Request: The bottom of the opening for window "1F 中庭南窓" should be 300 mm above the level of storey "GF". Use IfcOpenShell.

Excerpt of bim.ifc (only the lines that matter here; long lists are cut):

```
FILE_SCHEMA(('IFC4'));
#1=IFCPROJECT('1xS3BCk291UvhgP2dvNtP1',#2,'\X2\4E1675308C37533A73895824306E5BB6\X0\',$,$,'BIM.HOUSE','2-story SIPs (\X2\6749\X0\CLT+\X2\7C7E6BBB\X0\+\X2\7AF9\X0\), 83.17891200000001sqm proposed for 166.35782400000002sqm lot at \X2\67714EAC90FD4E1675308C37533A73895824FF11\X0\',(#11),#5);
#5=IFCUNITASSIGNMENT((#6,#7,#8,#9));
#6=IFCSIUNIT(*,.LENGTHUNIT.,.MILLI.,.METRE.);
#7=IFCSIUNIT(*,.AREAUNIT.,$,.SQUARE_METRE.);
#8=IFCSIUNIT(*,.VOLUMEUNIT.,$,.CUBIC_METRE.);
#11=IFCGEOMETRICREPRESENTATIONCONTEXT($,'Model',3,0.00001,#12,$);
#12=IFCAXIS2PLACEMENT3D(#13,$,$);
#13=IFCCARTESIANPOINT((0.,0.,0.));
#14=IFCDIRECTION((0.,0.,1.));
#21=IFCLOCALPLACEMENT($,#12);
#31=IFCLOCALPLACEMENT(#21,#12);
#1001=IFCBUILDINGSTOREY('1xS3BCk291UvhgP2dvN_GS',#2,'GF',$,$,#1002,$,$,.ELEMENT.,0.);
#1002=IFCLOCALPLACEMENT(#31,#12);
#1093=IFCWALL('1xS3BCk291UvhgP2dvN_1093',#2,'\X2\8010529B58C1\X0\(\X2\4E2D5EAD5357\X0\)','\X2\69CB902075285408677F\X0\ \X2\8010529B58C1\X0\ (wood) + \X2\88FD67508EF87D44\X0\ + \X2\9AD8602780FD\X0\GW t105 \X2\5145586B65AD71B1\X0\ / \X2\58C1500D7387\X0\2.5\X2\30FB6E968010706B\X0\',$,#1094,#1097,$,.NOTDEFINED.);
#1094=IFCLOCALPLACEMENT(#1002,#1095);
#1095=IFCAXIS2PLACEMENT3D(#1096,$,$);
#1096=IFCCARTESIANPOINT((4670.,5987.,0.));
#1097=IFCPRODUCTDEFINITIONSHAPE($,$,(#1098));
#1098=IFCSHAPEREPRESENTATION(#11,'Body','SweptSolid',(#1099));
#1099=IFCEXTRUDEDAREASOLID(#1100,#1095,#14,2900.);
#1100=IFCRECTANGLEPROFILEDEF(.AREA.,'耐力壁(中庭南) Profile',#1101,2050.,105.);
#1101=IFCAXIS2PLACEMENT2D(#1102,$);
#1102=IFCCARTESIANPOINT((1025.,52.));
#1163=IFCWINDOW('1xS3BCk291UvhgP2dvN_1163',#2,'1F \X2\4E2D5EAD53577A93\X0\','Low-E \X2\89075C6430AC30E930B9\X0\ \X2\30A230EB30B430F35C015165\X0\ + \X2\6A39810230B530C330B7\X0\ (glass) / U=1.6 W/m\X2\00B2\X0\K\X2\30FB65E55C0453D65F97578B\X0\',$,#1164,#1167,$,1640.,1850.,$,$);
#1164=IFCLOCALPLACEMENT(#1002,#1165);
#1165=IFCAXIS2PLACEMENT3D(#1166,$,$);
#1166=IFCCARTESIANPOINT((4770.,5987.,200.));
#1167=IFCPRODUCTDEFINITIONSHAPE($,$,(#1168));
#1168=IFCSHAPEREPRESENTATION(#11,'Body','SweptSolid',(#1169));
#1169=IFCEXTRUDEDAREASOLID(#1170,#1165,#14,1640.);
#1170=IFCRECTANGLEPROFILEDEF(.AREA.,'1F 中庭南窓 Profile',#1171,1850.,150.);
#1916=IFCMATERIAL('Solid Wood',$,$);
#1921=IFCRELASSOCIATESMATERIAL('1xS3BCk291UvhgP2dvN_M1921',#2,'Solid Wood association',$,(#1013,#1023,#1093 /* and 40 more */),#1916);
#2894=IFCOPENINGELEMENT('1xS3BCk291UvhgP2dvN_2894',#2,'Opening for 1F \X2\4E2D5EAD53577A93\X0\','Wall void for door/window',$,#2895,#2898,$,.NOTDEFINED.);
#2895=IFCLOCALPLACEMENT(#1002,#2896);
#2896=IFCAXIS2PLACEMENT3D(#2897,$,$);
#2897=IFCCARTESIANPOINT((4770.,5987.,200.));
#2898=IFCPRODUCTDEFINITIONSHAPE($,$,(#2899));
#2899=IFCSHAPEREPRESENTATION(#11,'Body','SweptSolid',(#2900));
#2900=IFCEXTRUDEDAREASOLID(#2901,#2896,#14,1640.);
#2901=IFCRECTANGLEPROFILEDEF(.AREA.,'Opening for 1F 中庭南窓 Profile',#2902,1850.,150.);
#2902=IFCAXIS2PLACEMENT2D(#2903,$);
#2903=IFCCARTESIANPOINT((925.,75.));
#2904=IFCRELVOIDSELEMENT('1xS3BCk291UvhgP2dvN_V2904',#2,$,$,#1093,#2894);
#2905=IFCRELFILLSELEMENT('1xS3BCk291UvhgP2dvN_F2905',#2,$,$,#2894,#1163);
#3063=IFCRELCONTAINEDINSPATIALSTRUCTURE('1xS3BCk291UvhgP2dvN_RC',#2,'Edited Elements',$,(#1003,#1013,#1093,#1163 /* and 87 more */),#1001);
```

```python
import numpy as np
import ifcopenshell
import ifcopenshell.api.geometry
import ifcopenshell.geom
import ifcopenshell.util.element
import ifcopenshell.util.placement
import ifcopenshell.util.shape
import ifcopenshell.util.unit

model = ifcopenshell.open("bim.ifc")
unit_scale = ifcopenshell.util.unit.calculate_unit_scale(model)

window = model.by_guid("1xS3BCk291UvhgP2dvN_1163")
opening = window.FillsVoids[0].RelatingOpeningElement
storey = ifcopenshell.util.element.get_container(window, ifc_class="IfcBuildingStorey")
level = ifcopenshell.util.placement.get_local_placement(storey.ObjectPlacement)[2, 3]

# The opening's origin need not be at the sill, so measure its lowest point.
shape = ifcopenshell.geom.create_shape(ifcopenshell.geom.settings(), opening)
bottom = ifcopenshell.util.shape.get_shape_bottom_elevation(shape, shape.geometry) / unit_scale
dz = level + 300.0 - bottom

shift = np.array([0.0, 0.0, dz])
# The window is not placed relative to its opening, so move both.
for product in (opening, window):
    matrix = ifcopenshell.util.placement.get_local_placement(product.ObjectPlacement)
    matrix[:3, 3] += shift
    ifcopenshell.api.geometry.edit_object_placement(model, product=product, matrix=matrix, is_si=False)

print(f"moved by {dz * unit_scale:+.3f} m")

model.write("bim_v2.ifc")
```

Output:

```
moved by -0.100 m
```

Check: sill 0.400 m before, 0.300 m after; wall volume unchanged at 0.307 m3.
